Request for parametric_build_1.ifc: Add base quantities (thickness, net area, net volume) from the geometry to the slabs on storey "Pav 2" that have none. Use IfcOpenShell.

First a look at what the model holds.

```python
import ifcopenshell
import ifcopenshell.util.element
import ifcopenshell.util.unit

model = ifcopenshell.open("parametric_build_1.ifc")
print(model.schema)
for unit_type in ("LENGTHUNIT", "AREAUNIT", "VOLUMEUNIT"):
    print(unit_type, ifcopenshell.util.unit.calculate_unit_scale(model, unit_type))
storey = next(s for s in model.by_type("IfcBuildingStorey") if s.Name == "Pav 2")
slabs = [e for e in ifcopenshell.util.element.get_decomposition(storey) if e.is_a("IfcSlab")]
for e in sorted(slabs, key=lambda e: e.id()):
    print(e.id(), e.is_a(), e.Name, list(ifcopenshell.util.element.get_psets(e, qtos_only=True)), sep=" | ")
```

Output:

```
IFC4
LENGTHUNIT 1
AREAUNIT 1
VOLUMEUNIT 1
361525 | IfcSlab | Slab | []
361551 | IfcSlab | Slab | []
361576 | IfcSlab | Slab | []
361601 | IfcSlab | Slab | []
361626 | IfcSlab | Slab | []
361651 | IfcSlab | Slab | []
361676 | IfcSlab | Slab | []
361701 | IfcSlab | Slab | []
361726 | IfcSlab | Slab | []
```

```python
import ifcopenshell
import ifcopenshell.api.pset
import ifcopenshell.geom
import ifcopenshell.util.element
import ifcopenshell.util.shape
import ifcopenshell.util.unit

model = ifcopenshell.open("parametric_build_1.ifc")
unit_scale = ifcopenshell.util.unit.calculate_unit_scale(model)
area_scale = ifcopenshell.util.unit.calculate_unit_scale(model, "AREAUNIT")
volume_scale = ifcopenshell.util.unit.calculate_unit_scale(model, "VOLUMEUNIT")
settings = ifcopenshell.geom.settings()

storey = next(s for s in model.by_type("IfcBuildingStorey") if s.Name == "Pav 2")
slabs = [e for e in ifcopenshell.util.element.get_decomposition(storey) if e.is_a("IfcSlab")]

for e in sorted(slabs, key=lambda e: e.id()):
    if ifcopenshell.util.element.get_psets(e, qtos_only=True, should_inherit=False):
        continue
    # Geometry comes back in metres, in the element's own axes.
    shape = ifcopenshell.geom.create_shape(settings, e)
    values = {
        "Width": ifcopenshell.util.shape.get_z(shape.geometry) / unit_scale,
        "NetArea": ifcopenshell.util.shape.get_footprint_area(shape.geometry) / area_scale,
        "NetVolume": ifcopenshell.util.shape.get_volume(shape.geometry) / volume_scale,
    }
    qto = ifcopenshell.api.pset.add_qto(model, product=e, name="Qto_SlabBaseQuantities")
    ifcopenshell.api.pset.edit_qto(model, qto=qto, properties=values)
    print(e.id(), {k: round(v, 3) for k, v in values.items()})

model.write("parametric_build_1_rev.ifc")
```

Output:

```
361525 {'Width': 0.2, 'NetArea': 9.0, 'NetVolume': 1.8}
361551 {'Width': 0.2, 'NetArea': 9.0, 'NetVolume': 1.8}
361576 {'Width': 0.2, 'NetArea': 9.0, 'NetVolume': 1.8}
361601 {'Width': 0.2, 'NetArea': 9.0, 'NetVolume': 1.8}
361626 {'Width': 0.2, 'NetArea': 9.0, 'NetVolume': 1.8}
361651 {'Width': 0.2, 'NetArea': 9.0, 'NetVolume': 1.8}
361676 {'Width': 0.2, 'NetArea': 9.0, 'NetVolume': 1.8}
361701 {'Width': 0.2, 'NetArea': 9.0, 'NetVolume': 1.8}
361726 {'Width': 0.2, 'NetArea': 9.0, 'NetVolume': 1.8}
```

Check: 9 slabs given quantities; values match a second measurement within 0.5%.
